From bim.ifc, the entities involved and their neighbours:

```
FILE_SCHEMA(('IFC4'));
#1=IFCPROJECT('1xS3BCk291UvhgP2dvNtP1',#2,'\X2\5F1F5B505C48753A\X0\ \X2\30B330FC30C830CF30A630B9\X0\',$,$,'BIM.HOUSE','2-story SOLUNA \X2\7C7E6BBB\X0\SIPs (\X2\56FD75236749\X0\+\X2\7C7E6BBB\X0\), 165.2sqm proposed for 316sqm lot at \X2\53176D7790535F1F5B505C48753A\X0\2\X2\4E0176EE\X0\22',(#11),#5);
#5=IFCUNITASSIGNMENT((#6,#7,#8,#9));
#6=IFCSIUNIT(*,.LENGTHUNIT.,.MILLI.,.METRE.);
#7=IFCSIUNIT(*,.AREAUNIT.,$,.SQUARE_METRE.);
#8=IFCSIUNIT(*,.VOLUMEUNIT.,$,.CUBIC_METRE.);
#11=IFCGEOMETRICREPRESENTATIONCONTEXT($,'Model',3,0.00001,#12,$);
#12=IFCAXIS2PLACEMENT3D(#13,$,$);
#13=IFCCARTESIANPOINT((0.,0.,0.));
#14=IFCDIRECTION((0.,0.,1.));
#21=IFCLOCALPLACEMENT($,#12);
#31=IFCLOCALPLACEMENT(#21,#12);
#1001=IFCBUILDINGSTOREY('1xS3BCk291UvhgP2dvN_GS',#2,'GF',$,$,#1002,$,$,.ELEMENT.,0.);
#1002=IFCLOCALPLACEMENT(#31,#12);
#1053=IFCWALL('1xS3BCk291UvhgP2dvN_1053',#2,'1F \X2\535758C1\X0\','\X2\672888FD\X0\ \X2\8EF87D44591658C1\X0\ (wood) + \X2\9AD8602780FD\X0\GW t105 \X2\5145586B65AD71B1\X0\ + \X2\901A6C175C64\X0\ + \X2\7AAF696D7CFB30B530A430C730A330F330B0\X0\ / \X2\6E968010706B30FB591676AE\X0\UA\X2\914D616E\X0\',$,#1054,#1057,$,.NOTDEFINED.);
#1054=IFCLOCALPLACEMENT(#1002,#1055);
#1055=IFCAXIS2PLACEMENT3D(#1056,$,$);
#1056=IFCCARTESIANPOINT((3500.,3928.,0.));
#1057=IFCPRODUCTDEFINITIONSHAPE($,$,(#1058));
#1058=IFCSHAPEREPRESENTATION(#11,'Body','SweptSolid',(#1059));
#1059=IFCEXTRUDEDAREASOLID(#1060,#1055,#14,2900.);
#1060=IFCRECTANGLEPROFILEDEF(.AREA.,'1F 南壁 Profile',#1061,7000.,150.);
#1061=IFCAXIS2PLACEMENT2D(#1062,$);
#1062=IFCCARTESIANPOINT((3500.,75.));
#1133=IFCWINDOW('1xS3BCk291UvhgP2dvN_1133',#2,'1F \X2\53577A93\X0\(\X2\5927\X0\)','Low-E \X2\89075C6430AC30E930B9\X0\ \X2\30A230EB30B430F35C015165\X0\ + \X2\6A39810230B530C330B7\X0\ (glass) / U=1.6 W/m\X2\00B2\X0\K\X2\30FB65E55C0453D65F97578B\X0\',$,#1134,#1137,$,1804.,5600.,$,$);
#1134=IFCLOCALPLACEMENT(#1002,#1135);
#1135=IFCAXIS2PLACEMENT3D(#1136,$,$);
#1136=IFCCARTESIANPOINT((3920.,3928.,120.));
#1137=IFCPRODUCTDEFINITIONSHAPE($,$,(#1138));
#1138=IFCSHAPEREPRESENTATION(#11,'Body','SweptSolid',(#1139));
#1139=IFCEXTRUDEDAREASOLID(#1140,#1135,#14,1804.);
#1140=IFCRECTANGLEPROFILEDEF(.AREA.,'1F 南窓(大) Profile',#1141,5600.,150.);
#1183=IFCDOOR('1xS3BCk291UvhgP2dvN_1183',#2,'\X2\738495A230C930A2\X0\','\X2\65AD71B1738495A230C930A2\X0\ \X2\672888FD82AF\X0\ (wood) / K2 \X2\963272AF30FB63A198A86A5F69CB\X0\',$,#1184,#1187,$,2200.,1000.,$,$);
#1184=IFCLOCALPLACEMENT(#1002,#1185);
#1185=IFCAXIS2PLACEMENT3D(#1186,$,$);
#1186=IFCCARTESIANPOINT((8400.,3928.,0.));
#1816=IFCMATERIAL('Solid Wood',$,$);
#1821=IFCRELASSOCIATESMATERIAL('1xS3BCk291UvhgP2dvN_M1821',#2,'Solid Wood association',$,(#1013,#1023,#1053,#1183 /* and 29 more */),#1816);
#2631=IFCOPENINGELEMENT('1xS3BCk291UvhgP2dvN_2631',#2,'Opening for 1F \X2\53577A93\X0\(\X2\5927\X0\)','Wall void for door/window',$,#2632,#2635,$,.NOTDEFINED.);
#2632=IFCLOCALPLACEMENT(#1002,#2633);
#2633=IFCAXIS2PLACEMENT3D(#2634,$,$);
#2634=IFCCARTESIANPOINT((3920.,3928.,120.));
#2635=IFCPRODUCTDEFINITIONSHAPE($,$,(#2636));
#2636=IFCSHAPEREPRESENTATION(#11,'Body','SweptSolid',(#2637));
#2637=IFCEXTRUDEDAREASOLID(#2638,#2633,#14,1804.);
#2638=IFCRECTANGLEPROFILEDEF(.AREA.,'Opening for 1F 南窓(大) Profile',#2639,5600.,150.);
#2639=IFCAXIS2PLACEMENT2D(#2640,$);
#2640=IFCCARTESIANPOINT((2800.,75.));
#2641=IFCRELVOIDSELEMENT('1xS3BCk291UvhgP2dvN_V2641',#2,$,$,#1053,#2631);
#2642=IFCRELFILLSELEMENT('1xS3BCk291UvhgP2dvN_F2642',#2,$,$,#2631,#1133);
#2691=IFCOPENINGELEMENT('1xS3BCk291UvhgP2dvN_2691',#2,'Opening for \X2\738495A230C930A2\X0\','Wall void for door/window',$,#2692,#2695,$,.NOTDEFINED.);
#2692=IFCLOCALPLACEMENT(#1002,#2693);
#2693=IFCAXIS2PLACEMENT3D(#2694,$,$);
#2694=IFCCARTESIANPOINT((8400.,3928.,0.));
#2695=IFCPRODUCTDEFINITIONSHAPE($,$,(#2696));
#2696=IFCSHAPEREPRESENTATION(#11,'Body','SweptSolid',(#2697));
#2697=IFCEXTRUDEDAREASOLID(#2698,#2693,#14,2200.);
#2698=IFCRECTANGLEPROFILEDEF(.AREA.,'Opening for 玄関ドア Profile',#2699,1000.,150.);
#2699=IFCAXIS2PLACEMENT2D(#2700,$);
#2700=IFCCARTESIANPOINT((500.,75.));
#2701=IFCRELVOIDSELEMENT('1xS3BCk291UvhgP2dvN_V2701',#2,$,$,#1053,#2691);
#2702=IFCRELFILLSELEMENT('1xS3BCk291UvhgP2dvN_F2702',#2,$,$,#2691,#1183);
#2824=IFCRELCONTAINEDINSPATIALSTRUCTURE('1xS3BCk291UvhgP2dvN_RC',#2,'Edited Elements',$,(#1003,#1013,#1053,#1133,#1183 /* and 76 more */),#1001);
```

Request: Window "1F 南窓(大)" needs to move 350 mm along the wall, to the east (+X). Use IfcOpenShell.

```python
import ifcopenshell
import ifcopenshell.api.geometry
import ifcopenshell.util.placement
import ifcopenshell.util.unit

model = ifcopenshell.open("bim.ifc")
unit_scale = ifcopenshell.util.unit.calculate_unit_scale(model)

window = model.by_guid("1xS3BCk291UvhgP2dvN_1133")
opening = window.FillsVoids[0].RelatingOpeningElement
wall = opening.VoidsElements[0].RelatingBuildingElement

wall_matrix = ifcopenshell.util.placement.get_local_placement(wall.ObjectPlacement)
shift = wall_matrix[:3, 0] * 0.35 / unit_scale
before = ifcopenshell.util.placement.get_local_placement(window.ObjectPlacement)[:3, 3].copy()

# The window is not placed relative to its opening, so move both.
for product in (opening, window):
    matrix = ifcopenshell.util.placement.get_local_placement(product.ObjectPlacement)
    matrix[:3, 3] += shift
    ifcopenshell.api.geometry.edit_object_placement(model, product=product, matrix=matrix, is_si=False)

after = ifcopenshell.util.placement.get_local_placement(window.ObjectPlacement)[:3, 3]
print("window moved by", (after - before).round(3) + 0.0)

model.write("bim-out.ifc")
```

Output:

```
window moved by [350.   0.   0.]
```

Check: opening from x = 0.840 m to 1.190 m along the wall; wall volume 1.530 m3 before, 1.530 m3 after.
